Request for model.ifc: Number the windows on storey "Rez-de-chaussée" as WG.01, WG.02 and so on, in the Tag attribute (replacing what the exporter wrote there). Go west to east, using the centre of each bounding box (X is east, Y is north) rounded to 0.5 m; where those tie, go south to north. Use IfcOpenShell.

First a look at what the model holds.

```python
import ifcopenshell
import ifcopenshell.util.element
import ifcopenshell.util.placement

model = ifcopenshell.open("model.ifc")
print(model.schema)
storey = next(s for s in model.by_type("IfcBuildingStorey") if s.Name == "Rez-de-chaussée")
windows = [e for e in ifcopenshell.util.element.get_decomposition(storey) if e.is_a("IfcWindow")]
for e in sorted(windows, key=lambda e: e.id()):
    origin = ifcopenshell.util.placement.get_local_placement(e.ObjectPlacement)[:3, 3]
    print(e.id(), e.Tag, e.Name, origin.round(2) + 0.0, sep=" | ")
```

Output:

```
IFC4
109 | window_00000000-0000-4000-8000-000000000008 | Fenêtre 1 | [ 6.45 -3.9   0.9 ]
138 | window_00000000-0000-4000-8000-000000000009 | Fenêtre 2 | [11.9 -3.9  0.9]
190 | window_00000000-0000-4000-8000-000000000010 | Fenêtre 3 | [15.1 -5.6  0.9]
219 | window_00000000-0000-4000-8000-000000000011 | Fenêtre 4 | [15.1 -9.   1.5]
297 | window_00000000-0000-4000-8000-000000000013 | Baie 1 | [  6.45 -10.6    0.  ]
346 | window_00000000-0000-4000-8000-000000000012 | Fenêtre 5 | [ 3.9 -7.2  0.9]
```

```python
import ifcopenshell
import ifcopenshell.geom
import ifcopenshell.util.element
import ifcopenshell.util.shape

model = ifcopenshell.open("model.ifc")
settings = ifcopenshell.geom.settings()
settings.set("use-world-coords", True)


def centre(element):
    shape = ifcopenshell.geom.create_shape(settings, element)
    return ifcopenshell.util.shape.get_bbox_centroid(shape.geometry)


storey = next(s for s in model.by_type("IfcBuildingStorey") if s.Name == "Rez-de-chaussée")
windows = [e for e in ifcopenshell.util.element.get_decomposition(storey) if e.is_a("IfcWindow")]

# Insertion points can sit at a corner or the storey origin, so sort by the geometry (in metres).
centres = {e: centre(e) for e in windows}
windows.sort(key=lambda e: (round(centres[e][0] / 0.5), centres[e][1]))

for i, e in enumerate(windows, start=1):
    number = f"WG.{i:02d}"
    e.Tag = number
    print(e.id(), number)

model.write("model_updated.ifc")
```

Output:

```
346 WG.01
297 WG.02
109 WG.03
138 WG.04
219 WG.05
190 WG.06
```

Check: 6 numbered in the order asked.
